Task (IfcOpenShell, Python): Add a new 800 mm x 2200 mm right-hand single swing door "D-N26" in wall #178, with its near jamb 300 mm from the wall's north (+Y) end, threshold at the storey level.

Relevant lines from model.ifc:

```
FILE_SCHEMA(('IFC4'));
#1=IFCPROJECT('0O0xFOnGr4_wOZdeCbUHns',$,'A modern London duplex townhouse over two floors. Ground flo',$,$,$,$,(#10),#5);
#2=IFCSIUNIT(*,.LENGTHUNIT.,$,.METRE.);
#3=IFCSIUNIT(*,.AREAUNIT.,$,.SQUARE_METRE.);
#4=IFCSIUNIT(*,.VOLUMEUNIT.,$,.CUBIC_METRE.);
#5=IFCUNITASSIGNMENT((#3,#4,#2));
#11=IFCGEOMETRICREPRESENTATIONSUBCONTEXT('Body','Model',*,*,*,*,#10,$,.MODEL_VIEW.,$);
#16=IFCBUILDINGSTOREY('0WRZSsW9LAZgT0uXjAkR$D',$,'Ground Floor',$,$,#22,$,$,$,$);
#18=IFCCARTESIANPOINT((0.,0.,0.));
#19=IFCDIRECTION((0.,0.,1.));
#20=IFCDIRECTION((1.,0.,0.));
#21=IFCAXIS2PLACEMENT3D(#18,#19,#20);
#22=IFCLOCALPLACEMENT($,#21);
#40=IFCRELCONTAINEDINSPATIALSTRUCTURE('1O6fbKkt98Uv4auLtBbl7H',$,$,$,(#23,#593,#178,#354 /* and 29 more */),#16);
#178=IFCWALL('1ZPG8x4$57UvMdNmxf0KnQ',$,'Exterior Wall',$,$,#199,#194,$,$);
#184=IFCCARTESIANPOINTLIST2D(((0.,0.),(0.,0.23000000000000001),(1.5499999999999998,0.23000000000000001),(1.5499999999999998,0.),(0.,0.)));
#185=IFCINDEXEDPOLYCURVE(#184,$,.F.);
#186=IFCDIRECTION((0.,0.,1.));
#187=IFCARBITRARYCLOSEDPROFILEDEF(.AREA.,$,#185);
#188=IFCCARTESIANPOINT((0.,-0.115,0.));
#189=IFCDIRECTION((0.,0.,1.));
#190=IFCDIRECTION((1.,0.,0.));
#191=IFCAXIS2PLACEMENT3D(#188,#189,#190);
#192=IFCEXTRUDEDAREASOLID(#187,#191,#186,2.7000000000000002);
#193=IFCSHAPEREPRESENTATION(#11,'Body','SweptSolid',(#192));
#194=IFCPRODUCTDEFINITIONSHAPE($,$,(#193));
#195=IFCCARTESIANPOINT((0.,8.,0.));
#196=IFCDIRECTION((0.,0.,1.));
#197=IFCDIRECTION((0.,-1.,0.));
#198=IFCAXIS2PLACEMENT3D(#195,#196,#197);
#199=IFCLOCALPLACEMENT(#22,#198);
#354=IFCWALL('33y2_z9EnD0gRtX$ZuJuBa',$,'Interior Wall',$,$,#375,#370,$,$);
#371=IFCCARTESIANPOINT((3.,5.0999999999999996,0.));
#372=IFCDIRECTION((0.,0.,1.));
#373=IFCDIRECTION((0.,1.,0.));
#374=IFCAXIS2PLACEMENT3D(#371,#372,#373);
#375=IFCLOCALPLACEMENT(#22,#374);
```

```python
import numpy as np
import ifcopenshell
import ifcopenshell.api.feature
import ifcopenshell.api.geometry
import ifcopenshell.api.root
import ifcopenshell.api.spatial
import ifcopenshell.geom
import ifcopenshell.util.element
import ifcopenshell.util.placement
import ifcopenshell.util.representation
import ifcopenshell.util.shape
import ifcopenshell.util.unit

model = ifcopenshell.open("model.ifc")
unit_scale = ifcopenshell.util.unit.calculate_unit_scale(model)
settings = ifcopenshell.geom.settings()


def volume(element):
    """Net volume in cubic metres, openings subtracted."""
    shape = ifcopenshell.geom.create_shape(settings, element)
    return ifcopenshell.util.shape.get_volume(shape.geometry)


wall = model.by_guid("1ZPG8x4$57UvMdNmxf0KnQ")
storey = ifcopenshell.util.element.get_container(wall, ifc_class="IfcBuildingStorey")
context = ifcopenshell.util.representation.get_context(model, "Model", "Body", "MODEL_VIEW")
before = volume(wall)

width, height, from_end, sill = 0.8, 2.2, 0.3, 0.0  # metres

# The wall runs along its own X axis, and the end named is its -X end.
wall_shape = ifcopenshell.geom.create_shape(settings, wall)
x, y, z = ifcopenshell.util.shape.get_vertices(wall_shape.geometry).T
start = x.min() + from_end
face, thickness = float(y.min()), float(y.max() - y.min())
wall_matrix = ifcopenshell.util.placement.get_local_placement(wall.ObjectPlacement)
level = ifcopenshell.util.placement.get_local_placement(storey.ObjectPlacement)[2, 3]


def in_wall(x, y):
    """Placement at x, y metres in the wall's axes, at sill height."""
    matrix = wall_matrix.copy()
    matrix[:, 3] = wall_matrix @ np.array([x / unit_scale, y / unit_scale, 0.0, 1.0])
    matrix[2, 3] = level + sill / unit_scale
    return matrix


# Opening: a box that overshoots both wall faces by 50 mm.
opening = ifcopenshell.api.root.create_entity(model, ifc_class="IfcOpeningElement", predefined_type="OPENING")
box = ifcopenshell.api.geometry.add_wall_representation(
    model, context=context, length=width, height=height, thickness=thickness + 0.1
)
ifcopenshell.api.geometry.assign_representation(model, product=opening, representation=box)
ifcopenshell.api.geometry.edit_object_placement(model, product=opening, matrix=in_wall(start, face - 0.05), is_si=False)
ifcopenshell.api.feature.add_feature(model, feature=opening, element=wall)

door = ifcopenshell.api.root.create_entity(model, ifc_class="IfcDoor", name="D-N26", predefined_type="DOOR")
door.OverallWidth, door.OverallHeight = width / unit_scale, height / unit_scale
door.OperationType = "SINGLE_SWING_RIGHT"
body = ifcopenshell.api.geometry.add_door_representation(
    model,
    context=context,
    overall_width=door.OverallWidth,
    overall_height=door.OverallHeight,
    operation_type="SINGLE_SWING_RIGHT",
    lining_properties={"LiningDepth": thickness / unit_scale, "ThresholdDepth": thickness / unit_scale},
)
ifcopenshell.api.geometry.assign_representation(model, product=door, representation=body)
ifcopenshell.api.spatial.assign_container(model, products=[door], relating_structure=storey)
ifcopenshell.api.feature.add_filling(model, opening=opening, element=door)

# The lining spans the wall, so the door starts at the wall face.
ifcopenshell.api.geometry.edit_object_placement(model, product=door, matrix=in_wall(start, face), is_si=False)

after = volume(wall)

print(f"wall volume {before:.3f} -> {after:.3f} m3")

model.write("model_rev.ifc")
```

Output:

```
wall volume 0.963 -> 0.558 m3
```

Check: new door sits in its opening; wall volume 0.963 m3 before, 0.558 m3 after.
